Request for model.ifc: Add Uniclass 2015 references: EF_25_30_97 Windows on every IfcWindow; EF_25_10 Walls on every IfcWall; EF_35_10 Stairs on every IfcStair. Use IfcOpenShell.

First a look at what the model holds.

```python
import ifcopenshell

model = ifcopenshell.open("model.ifc")
print(model.schema)
print("classifications:", [c.Name for c in model.by_type("IfcClassification")])
for ifc_class in ("IfcDoor", "IfcRoof", "IfcStair", "IfcWall", "IfcWindow"):
    print(ifc_class, len(model.by_type(ifc_class)))
```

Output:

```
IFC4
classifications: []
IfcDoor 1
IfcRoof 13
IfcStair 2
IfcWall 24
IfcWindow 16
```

```python
import ifcopenshell
import ifcopenshell.api.classification

model = ifcopenshell.open("model.ifc")

system = ifcopenshell.api.classification.add_classification(model, classification="Uniclass 2015")

codes = {
    "IfcWindow": ("EF_25_30_97", "Windows"),
    "IfcWall": ("EF_25_10", "Walls"),
    "IfcStair": ("EF_35_10", "Stairs"),
}
for ifc_class, (code, name) in codes.items():
    products = model.by_type(ifc_class)
    ifcopenshell.api.classification.add_reference(
        model, products=products, classification=system, identification=code, name=name
    )
    print(code, len(products))

model.write("model_updated.ifc")
```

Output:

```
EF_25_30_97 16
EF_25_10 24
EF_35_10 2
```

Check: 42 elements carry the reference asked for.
